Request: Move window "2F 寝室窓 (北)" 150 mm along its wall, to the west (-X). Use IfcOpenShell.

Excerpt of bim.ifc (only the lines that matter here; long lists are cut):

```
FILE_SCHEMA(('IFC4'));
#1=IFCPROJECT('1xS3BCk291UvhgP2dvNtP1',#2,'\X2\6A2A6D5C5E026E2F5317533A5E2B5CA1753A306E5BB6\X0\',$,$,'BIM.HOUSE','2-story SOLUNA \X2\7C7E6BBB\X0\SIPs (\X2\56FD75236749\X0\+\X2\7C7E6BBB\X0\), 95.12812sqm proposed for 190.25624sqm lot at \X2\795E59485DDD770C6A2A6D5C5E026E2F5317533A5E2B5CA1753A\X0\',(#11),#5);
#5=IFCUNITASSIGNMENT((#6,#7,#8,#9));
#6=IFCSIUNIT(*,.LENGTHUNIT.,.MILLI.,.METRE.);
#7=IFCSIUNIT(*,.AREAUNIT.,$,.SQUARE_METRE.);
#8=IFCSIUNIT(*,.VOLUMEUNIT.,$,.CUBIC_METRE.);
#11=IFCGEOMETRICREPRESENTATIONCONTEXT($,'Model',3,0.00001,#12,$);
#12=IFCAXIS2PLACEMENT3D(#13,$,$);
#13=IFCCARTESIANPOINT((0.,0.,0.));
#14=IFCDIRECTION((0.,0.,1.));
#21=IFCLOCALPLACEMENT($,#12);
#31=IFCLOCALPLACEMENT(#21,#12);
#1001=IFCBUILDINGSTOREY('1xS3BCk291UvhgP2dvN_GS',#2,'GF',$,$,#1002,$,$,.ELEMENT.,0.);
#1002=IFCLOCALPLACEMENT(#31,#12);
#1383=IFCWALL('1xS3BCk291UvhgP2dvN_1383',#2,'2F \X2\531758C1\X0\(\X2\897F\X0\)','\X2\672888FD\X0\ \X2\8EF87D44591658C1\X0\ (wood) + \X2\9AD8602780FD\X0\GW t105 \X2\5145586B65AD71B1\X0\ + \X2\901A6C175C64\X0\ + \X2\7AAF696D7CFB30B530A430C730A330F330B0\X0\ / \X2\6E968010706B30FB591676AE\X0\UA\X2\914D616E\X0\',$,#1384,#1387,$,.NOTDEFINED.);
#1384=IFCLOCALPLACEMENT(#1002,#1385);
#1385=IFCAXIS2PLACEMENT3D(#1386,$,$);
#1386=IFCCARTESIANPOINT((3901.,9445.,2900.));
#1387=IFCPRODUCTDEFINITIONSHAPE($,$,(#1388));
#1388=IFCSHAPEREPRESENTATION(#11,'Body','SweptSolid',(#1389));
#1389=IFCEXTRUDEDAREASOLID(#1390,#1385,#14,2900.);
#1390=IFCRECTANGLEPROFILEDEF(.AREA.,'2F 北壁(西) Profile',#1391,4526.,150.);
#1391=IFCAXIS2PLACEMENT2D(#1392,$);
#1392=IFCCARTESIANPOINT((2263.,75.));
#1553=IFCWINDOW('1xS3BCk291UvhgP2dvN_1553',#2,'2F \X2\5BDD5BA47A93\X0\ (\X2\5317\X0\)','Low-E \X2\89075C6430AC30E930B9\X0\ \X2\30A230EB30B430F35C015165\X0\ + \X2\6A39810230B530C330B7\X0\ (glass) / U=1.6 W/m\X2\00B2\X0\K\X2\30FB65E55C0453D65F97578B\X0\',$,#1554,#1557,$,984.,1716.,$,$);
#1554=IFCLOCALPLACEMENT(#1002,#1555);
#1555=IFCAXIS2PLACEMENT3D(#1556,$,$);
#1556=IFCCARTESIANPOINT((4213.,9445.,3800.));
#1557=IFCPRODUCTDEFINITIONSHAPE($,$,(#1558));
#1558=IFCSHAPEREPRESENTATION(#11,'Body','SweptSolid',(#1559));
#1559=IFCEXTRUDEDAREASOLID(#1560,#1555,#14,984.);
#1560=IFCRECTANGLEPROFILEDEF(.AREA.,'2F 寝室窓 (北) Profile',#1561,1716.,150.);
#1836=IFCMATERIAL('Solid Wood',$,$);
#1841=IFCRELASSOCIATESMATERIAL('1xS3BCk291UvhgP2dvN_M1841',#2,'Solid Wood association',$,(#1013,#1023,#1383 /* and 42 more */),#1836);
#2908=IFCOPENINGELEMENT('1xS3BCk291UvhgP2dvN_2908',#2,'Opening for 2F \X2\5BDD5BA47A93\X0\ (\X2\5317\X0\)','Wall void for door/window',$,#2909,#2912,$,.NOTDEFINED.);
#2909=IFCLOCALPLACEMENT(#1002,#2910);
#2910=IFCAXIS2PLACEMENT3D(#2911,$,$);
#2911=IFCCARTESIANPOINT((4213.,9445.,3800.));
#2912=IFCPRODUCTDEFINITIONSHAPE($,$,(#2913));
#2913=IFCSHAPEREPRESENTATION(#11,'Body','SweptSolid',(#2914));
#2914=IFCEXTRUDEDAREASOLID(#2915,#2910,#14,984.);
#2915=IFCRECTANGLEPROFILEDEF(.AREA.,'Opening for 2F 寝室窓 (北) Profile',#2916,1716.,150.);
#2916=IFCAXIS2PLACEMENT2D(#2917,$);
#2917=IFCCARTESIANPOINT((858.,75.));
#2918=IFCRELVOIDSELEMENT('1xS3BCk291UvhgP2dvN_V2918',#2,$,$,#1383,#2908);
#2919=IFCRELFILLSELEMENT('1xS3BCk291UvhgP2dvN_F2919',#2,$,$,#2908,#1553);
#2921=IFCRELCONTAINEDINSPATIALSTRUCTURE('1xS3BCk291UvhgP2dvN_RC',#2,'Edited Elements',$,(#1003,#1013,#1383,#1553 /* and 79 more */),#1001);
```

```python
import ifcopenshell
import ifcopenshell.api.geometry
import ifcopenshell.util.placement
import ifcopenshell.util.unit

model = ifcopenshell.open("bim.ifc")
unit_scale = ifcopenshell.util.unit.calculate_unit_scale(model)

window = model.by_guid("1xS3BCk291UvhgP2dvN_1553")
opening = window.FillsVoids[0].RelatingOpeningElement
wall = opening.VoidsElements[0].RelatingBuildingElement

wall_matrix = ifcopenshell.util.placement.get_local_placement(wall.ObjectPlacement)
shift = wall_matrix[:3, 0] * -0.15 / unit_scale
before = ifcopenshell.util.placement.get_local_placement(window.ObjectPlacement)[:3, 3].copy()

# The window is not placed relative to its opening, so move both.
for product in (opening, window):
    matrix = ifcopenshell.util.placement.get_local_placement(product.ObjectPlacement)
    matrix[:3, 3] += shift
    ifcopenshell.api.geometry.edit_object_placement(model, product=product, matrix=matrix, is_si=False)

after = ifcopenshell.util.placement.get_local_placement(window.ObjectPlacement)[:3, 3]
print("window moved by", (after - before).round(3) + 0.0)

model.write("bim_edited.ifc")
```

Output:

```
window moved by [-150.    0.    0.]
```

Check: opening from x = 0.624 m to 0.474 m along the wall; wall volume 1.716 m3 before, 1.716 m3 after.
